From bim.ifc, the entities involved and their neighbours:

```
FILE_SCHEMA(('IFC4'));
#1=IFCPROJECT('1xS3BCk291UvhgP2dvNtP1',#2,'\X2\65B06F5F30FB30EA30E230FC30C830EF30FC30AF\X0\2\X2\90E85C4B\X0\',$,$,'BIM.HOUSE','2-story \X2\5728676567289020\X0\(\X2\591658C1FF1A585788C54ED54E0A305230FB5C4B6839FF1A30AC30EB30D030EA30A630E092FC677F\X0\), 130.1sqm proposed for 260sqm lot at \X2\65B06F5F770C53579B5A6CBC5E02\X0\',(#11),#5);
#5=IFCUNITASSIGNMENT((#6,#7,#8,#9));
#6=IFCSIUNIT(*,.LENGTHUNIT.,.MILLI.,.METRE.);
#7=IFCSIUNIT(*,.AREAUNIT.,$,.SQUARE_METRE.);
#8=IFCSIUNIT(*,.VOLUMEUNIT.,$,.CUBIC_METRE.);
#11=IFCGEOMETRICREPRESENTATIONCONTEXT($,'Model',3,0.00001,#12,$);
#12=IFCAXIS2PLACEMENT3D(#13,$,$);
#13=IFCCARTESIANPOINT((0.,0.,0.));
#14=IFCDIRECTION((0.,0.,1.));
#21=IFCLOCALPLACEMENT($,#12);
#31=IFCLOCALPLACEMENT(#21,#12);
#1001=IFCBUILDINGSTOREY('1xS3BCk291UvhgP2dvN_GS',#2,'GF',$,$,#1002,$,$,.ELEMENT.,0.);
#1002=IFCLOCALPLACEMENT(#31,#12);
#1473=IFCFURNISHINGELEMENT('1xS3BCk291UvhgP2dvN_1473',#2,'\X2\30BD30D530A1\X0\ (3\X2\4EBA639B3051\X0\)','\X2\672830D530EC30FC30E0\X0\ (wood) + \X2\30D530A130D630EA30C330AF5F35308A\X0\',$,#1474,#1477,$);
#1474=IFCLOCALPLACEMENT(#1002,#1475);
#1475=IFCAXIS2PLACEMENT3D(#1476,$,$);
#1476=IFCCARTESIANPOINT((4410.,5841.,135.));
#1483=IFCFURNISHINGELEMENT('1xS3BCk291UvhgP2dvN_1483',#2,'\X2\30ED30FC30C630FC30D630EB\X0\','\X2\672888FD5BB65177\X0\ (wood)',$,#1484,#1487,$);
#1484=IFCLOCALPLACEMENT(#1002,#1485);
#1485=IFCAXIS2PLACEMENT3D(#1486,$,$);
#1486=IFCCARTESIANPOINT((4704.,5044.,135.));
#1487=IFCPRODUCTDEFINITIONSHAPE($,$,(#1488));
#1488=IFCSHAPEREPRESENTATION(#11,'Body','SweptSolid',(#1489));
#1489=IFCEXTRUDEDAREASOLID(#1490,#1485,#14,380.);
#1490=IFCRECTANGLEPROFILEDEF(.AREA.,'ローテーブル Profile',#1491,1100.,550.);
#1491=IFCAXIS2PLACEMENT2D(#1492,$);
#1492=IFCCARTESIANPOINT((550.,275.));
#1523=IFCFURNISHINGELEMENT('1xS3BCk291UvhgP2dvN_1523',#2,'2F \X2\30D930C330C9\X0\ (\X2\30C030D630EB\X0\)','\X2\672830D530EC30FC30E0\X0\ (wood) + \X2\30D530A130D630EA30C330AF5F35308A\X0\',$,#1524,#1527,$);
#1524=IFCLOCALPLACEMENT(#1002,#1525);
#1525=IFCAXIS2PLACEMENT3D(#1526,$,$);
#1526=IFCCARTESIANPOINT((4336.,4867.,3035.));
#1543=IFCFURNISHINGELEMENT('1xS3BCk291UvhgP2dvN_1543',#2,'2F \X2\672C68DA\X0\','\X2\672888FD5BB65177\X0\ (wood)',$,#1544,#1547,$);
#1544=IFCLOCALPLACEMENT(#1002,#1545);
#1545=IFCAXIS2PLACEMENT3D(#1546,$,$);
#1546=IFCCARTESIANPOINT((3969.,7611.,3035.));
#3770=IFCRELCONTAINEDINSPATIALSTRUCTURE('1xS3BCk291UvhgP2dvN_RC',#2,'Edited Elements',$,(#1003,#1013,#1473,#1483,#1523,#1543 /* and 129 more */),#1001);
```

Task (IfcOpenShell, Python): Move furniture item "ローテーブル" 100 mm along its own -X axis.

```python
import ifcopenshell
import ifcopenshell.api.geometry
import ifcopenshell.util.placement
import ifcopenshell.util.unit

model = ifcopenshell.open("bim.ifc")
unit_scale = ifcopenshell.util.unit.calculate_unit_scale(model)

item = model.by_guid("1xS3BCk291UvhgP2dvN_1483")
matrix = ifcopenshell.util.placement.get_local_placement(item.ObjectPlacement)
matrix[:3, 3] -= matrix[:3, 0] * 0.1 / unit_scale
ifcopenshell.api.geometry.edit_object_placement(model, product=item, matrix=matrix, is_si=False)

print(ifcopenshell.util.placement.get_local_placement(item.ObjectPlacement).round(3) + 0.0)

model.write("bim-out.ifc")
```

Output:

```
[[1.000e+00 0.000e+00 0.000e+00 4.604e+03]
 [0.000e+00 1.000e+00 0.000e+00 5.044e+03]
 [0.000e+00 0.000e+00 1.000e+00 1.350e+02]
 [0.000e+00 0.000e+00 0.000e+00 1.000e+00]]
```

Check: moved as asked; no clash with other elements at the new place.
